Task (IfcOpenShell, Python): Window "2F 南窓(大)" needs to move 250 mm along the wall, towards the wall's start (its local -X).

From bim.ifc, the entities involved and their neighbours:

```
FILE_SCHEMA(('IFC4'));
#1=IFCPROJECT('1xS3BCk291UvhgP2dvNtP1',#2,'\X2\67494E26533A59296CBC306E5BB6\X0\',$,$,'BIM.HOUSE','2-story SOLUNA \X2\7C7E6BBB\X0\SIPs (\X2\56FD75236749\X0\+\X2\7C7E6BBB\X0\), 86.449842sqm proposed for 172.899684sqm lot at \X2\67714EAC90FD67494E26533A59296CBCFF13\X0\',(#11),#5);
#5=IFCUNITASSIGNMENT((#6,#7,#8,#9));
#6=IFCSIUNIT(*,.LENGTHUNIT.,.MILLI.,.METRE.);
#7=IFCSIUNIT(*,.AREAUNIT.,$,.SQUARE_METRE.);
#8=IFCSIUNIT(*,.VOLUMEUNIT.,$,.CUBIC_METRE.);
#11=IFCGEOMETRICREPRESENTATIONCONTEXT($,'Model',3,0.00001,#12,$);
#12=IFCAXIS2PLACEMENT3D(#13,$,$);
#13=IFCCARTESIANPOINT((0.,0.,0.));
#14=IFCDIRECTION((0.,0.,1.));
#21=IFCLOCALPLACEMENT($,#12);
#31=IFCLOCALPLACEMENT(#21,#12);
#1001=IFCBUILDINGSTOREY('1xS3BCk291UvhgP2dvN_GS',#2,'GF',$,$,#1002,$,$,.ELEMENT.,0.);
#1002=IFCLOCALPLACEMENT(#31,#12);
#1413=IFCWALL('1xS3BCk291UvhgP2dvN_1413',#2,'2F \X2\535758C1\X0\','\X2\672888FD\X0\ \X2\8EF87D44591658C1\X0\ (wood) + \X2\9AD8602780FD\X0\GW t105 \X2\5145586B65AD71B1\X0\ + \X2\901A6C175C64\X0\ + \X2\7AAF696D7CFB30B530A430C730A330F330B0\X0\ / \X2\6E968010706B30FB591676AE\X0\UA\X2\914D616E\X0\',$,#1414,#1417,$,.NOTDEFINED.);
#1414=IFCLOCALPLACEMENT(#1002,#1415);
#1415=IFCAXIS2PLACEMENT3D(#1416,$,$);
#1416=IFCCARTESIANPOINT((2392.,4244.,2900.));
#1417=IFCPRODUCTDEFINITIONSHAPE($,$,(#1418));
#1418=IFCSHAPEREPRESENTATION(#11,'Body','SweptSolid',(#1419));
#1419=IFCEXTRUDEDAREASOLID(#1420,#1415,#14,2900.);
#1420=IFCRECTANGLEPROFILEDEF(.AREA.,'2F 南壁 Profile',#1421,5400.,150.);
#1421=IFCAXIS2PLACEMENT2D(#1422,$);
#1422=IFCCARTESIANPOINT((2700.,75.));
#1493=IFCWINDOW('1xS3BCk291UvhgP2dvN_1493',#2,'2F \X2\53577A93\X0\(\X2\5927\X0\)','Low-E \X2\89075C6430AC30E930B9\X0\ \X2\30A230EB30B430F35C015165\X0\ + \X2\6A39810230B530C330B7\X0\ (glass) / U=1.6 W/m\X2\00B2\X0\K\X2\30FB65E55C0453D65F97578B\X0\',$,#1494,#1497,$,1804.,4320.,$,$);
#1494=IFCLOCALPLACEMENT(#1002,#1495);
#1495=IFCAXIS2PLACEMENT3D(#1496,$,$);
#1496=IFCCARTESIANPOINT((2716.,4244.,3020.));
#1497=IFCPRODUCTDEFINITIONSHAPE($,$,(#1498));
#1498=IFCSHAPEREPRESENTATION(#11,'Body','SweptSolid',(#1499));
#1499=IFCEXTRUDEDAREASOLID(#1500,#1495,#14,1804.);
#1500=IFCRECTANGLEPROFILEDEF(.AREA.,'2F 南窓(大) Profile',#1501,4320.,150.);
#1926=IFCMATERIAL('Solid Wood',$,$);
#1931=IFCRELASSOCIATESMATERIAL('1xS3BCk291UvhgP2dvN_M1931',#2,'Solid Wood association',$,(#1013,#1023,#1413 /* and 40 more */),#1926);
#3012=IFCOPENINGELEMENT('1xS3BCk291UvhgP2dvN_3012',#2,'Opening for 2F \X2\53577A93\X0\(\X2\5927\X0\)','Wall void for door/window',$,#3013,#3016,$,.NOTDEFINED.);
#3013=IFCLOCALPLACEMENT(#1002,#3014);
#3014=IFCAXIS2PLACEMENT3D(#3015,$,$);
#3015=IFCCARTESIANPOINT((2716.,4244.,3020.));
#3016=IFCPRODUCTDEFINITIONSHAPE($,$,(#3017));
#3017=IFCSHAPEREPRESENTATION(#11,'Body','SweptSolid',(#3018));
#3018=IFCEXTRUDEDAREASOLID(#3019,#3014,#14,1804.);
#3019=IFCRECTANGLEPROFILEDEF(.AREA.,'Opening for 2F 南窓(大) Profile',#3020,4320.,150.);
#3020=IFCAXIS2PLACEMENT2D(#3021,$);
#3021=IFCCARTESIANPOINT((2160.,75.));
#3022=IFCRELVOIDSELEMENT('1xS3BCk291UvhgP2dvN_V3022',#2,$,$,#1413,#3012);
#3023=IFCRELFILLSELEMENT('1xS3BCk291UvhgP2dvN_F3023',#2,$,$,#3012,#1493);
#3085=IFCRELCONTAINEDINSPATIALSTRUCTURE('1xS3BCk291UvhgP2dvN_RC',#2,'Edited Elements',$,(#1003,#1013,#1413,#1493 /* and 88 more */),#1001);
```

```python
import ifcopenshell
import ifcopenshell.api.geometry
import ifcopenshell.util.placement

model = ifcopenshell.open("bim.ifc")

window = model.by_guid("1xS3BCk291UvhgP2dvN_1493")
opening = window.FillsVoids[0].RelatingOpeningElement
wall = opening.VoidsElements[0].RelatingBuildingElement

wall_matrix = ifcopenshell.util.placement.get_local_placement(wall.ObjectPlacement)
shift = wall_matrix[:3, 0] * -250.0
before = ifcopenshell.util.placement.get_local_placement(window.ObjectPlacement)[:3, 3].copy()

# The window is not placed relative to its opening, so move both.
for product in (opening, window):
    matrix = ifcopenshell.util.placement.get_local_placement(product.ObjectPlacement)
    matrix[:3, 3] += shift
    ifcopenshell.api.geometry.edit_object_placement(model, product=product, matrix=matrix, is_si=False)

after = ifcopenshell.util.placement.get_local_placement(window.ObjectPlacement)[:3, 3]
print("window moved by", (after - before).round(3) + 0.0)

model.write("bim_updated.ifc")
```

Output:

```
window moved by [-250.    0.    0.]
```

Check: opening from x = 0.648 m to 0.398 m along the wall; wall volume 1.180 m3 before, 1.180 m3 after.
